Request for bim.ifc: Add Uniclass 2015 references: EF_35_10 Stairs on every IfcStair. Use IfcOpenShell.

First a look at what the model holds.

```python
import ifcopenshell

model = ifcopenshell.open("bim.ifc")
print(model.schema)
print("classifications:", [c.Name for c in model.by_type("IfcClassification")])
for ifc_class in ("IfcDoor", "IfcRoof", "IfcStair", "IfcWall", "IfcWindow"):
    print(ifc_class, len(model.by_type(ifc_class)))
```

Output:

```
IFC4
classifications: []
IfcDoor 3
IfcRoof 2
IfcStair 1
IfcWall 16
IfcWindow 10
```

```python
import ifcopenshell
import ifcopenshell.api.classification

model = ifcopenshell.open("bim.ifc")

system = ifcopenshell.api.classification.add_classification(model, classification="Uniclass 2015")

codes = {
    "IfcStair": ("EF_35_10", "Stairs"),
}
for ifc_class, (code, name) in codes.items():
    products = model.by_type(ifc_class)
    ifcopenshell.api.classification.add_reference(
        model, products=products, classification=system, identification=code, name=name
    )
    print(code, len(products))

model.write("bim_edited.ifc")
```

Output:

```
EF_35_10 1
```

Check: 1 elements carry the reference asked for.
